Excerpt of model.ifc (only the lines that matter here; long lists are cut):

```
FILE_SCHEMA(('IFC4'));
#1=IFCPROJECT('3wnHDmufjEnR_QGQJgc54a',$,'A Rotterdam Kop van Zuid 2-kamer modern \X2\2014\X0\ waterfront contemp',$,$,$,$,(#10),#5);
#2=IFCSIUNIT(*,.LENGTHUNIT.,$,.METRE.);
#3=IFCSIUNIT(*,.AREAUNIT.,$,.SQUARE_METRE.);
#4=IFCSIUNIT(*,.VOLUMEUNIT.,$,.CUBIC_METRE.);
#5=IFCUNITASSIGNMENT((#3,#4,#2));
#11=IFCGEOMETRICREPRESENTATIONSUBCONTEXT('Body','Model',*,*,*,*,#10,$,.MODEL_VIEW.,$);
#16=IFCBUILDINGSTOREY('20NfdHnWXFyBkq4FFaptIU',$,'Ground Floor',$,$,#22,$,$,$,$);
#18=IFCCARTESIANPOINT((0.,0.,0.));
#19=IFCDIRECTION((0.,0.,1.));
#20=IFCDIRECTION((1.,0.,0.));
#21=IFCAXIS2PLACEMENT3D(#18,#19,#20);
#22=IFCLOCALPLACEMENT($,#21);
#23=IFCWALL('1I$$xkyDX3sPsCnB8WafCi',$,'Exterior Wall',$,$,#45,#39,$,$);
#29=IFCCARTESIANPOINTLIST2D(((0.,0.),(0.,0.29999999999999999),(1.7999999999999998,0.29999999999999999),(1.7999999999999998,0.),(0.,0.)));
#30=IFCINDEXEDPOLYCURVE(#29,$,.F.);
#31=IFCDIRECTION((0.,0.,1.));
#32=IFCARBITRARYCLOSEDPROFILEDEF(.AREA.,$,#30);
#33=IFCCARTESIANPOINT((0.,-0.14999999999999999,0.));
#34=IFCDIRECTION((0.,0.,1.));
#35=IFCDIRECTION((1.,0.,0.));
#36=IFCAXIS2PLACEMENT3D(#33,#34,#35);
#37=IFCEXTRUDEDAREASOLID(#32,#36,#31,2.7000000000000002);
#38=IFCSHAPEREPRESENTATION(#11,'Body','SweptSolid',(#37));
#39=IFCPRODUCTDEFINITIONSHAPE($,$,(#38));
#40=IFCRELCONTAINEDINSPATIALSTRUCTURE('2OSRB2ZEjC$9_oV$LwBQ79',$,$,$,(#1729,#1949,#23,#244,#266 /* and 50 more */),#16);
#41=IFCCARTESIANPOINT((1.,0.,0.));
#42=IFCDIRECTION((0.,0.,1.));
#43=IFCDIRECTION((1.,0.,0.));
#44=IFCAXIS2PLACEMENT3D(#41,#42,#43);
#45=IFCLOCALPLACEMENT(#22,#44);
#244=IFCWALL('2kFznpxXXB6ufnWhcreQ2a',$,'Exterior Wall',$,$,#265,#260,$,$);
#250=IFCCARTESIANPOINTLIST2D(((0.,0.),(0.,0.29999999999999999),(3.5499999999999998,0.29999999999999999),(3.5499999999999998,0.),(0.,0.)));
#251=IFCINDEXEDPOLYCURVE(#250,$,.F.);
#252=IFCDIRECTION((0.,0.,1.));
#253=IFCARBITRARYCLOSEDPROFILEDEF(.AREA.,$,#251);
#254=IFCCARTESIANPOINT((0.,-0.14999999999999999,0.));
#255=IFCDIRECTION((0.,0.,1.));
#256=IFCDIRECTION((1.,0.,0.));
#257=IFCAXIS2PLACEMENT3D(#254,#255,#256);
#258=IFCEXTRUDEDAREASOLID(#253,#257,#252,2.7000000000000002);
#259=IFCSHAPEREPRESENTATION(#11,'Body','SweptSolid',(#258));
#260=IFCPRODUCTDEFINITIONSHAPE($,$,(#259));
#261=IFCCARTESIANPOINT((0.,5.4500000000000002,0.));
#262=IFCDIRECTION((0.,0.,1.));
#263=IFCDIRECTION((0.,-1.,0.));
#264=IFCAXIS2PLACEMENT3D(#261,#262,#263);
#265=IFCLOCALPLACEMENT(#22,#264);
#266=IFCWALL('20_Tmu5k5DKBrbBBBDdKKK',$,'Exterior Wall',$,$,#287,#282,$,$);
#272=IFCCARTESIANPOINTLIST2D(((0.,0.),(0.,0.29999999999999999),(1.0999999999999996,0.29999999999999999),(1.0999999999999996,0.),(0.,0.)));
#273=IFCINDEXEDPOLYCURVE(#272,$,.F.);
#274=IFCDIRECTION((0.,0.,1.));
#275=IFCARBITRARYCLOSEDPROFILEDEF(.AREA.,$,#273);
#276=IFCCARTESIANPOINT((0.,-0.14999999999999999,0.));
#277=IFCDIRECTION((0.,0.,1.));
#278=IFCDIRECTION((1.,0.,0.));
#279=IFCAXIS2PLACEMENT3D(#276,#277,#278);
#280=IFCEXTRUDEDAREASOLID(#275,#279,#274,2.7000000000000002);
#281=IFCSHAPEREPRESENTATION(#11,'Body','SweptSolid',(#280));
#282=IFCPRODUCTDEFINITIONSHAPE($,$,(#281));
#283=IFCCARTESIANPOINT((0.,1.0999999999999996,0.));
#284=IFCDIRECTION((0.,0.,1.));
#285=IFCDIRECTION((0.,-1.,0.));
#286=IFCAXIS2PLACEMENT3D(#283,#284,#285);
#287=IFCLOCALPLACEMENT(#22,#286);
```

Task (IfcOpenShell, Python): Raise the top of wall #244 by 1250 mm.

```python
import ifcopenshell
import ifcopenshell.geom
import ifcopenshell.util.representation
import ifcopenshell.util.shape
import ifcopenshell.util.unit

model = ifcopenshell.open("model.ifc")
unit_scale = ifcopenshell.util.unit.calculate_unit_scale(model)
settings = ifcopenshell.geom.settings()


def volume(element):
    """Net volume in cubic metres, openings subtracted."""
    shape = ifcopenshell.geom.create_shape(settings, element)
    return ifcopenshell.util.shape.get_volume(shape.geometry)


wall = model.by_id(244)
before = volume(wall)

body = ifcopenshell.util.representation.get_representation(wall, "Model", "Body")
solid = body.Items[0]
old_height = solid.Depth
solid.Depth += 1.25 / unit_scale
after = volume(wall)

print(f"height {old_height:g} -> {solid.Depth:g}, volume {before:.3f} -> {after:.3f} m3")

model.write("model_rev.ifc")
```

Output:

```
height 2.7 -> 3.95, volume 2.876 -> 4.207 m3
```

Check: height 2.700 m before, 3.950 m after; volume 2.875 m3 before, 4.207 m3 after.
